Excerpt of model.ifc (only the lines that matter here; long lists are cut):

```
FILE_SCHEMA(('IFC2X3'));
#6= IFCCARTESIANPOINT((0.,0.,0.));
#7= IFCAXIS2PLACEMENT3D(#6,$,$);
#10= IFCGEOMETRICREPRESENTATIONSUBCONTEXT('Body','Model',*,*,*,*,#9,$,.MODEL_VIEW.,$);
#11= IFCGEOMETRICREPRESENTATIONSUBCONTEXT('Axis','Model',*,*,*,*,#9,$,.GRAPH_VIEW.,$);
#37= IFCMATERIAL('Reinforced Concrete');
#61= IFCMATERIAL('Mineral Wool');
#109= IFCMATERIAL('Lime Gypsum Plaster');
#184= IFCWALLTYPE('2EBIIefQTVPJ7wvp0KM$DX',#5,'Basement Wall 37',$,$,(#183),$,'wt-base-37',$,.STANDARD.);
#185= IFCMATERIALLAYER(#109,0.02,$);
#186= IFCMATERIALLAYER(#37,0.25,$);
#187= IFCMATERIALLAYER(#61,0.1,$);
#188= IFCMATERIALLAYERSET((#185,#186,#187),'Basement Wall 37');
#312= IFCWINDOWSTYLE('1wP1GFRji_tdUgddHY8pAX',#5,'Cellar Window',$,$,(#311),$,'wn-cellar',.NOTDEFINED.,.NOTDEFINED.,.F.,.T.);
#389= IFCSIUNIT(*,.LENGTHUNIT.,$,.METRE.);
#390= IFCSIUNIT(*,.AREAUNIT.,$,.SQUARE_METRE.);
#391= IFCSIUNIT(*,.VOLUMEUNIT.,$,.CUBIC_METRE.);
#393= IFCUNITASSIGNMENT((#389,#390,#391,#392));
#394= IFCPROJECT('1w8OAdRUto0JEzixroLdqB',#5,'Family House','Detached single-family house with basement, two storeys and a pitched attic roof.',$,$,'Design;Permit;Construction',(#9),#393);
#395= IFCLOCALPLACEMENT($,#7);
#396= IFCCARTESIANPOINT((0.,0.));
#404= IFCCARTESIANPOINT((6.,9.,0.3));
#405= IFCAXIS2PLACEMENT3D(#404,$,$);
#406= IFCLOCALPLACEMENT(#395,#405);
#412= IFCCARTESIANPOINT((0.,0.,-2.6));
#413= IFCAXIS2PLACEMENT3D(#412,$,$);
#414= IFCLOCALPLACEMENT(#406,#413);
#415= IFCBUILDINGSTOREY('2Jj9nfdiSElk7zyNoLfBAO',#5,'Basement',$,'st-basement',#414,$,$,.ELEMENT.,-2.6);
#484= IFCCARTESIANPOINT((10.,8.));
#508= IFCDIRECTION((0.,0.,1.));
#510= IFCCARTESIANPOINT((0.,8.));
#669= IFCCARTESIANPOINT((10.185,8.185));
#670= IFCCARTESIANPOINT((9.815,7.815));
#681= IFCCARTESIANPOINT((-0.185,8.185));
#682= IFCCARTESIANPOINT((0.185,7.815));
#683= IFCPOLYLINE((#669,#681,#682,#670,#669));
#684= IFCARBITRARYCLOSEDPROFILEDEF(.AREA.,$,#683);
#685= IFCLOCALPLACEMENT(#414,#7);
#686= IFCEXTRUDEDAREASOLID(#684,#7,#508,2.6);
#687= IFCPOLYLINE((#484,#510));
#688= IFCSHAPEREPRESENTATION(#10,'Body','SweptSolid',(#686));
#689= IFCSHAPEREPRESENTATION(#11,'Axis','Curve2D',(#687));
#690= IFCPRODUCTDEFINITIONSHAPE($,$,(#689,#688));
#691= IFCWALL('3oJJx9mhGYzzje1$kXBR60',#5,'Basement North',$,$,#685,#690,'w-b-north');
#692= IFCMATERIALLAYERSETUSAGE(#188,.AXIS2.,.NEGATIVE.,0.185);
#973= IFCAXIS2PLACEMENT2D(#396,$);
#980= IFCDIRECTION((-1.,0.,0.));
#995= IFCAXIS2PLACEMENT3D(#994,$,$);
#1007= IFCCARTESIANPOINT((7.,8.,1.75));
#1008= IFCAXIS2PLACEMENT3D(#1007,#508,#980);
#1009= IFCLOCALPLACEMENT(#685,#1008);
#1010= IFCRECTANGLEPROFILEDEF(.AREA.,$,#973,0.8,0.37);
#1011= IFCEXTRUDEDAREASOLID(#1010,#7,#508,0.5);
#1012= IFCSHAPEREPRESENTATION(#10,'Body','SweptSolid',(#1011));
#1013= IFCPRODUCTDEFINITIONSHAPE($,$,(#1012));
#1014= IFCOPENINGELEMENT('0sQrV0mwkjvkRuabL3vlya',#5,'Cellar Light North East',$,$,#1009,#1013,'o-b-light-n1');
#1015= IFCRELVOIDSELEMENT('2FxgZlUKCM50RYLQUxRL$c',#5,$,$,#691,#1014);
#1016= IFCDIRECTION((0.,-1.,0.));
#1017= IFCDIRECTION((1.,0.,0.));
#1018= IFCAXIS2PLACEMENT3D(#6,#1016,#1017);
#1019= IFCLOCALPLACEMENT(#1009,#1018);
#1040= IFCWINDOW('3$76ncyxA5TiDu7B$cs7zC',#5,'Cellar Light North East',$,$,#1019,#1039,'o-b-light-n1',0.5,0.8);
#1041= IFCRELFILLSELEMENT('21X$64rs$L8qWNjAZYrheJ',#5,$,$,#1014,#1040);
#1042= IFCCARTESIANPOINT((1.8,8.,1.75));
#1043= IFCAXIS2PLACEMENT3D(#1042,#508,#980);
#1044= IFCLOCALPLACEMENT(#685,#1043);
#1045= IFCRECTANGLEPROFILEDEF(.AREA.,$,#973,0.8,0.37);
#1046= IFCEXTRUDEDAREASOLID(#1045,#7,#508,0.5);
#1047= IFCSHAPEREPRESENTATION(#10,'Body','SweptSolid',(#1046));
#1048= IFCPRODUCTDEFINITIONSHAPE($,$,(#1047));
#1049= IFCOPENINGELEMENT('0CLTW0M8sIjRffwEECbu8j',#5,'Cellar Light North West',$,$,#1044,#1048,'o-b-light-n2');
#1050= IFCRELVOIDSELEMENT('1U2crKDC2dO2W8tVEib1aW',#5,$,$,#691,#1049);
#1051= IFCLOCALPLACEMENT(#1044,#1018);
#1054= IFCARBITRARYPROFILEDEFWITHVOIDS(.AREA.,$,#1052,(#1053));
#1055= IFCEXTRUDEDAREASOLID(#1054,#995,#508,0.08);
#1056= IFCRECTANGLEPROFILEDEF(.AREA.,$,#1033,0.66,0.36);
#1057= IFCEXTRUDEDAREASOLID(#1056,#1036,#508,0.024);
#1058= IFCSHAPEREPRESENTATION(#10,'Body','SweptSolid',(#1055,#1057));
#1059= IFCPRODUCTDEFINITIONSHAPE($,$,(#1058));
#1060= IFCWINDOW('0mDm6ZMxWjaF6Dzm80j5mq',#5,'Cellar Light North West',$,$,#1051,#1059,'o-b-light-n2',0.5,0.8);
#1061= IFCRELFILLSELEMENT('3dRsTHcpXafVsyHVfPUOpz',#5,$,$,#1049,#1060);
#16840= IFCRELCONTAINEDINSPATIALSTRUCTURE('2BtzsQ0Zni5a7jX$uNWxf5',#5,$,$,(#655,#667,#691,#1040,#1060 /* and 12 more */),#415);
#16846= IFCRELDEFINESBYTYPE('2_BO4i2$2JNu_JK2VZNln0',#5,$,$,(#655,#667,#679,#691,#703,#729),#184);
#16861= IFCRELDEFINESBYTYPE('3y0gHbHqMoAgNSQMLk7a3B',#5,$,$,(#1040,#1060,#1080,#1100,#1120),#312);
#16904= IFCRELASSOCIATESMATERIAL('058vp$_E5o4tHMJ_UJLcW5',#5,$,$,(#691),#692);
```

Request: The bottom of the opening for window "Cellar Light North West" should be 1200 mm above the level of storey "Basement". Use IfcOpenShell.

```python
import numpy as np
import ifcopenshell
import ifcopenshell.api.geometry
import ifcopenshell.geom
import ifcopenshell.util.element
import ifcopenshell.util.placement
import ifcopenshell.util.shape
import ifcopenshell.util.unit

model = ifcopenshell.open("model.ifc")
unit_scale = ifcopenshell.util.unit.calculate_unit_scale(model)

window = model.by_guid("0mDm6ZMxWjaF6Dzm80j5mq")
opening = window.FillsVoids[0].RelatingOpeningElement
storey = ifcopenshell.util.element.get_container(window, ifc_class="IfcBuildingStorey")
level = ifcopenshell.util.placement.get_local_placement(storey.ObjectPlacement)[2, 3]

# The opening's origin need not be at the sill, so measure its lowest point.
shape = ifcopenshell.geom.create_shape(ifcopenshell.geom.settings(), opening)
bottom = ifcopenshell.util.shape.get_shape_bottom_elevation(shape, shape.geometry) / unit_scale
dz = level + 1.2 / unit_scale - bottom

shift = np.array([0.0, 0.0, dz])
# The window is placed relative to its opening, so it follows when the opening moves.
matrix = ifcopenshell.util.placement.get_local_placement(opening.ObjectPlacement)
matrix[:3, 3] += shift
ifcopenshell.api.geometry.edit_object_placement(
    model, product=opening, matrix=matrix, is_si=False, should_transform_children=True
)

print(f"moved by {dz * unit_scale:+.3f} m")

model.write("model_rev.ifc")
```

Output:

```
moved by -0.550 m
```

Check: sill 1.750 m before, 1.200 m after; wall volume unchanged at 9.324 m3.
